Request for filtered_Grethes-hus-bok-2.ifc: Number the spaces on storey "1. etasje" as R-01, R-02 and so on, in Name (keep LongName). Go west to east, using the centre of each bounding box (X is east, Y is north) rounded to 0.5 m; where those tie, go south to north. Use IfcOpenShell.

First a look at what the model holds.

```python
import ifcopenshell
import ifcopenshell.util.element
import ifcopenshell.util.placement

model = ifcopenshell.open("filtered_Grethes-hus-bok-2.ifc")
print(model.schema)
storey = next(s for s in model.by_type("IfcBuildingStorey") if s.Name == "1. etasje")
spaces = [e for e in ifcopenshell.util.element.get_decomposition(storey) if e.is_a("IfcSpace")]
for e in sorted(spaces, key=lambda e: e.id()):
    origin = ifcopenshell.util.placement.get_local_placement(e.ObjectPlacement)[:3, 3]
    print(e.id(), e.Name, e.LongName, origin.round(2) + 0.0, sep=" | ")
```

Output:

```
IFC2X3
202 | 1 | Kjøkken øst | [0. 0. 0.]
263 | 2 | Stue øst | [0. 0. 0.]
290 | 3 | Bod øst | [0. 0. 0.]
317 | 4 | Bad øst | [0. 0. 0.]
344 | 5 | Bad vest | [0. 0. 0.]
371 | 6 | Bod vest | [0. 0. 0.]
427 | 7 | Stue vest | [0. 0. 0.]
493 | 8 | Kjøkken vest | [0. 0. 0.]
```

```python
import ifcopenshell
import ifcopenshell.geom
import ifcopenshell.util.element
import ifcopenshell.util.shape

model = ifcopenshell.open("filtered_Grethes-hus-bok-2.ifc")
settings = ifcopenshell.geom.settings()
settings.set("use-world-coords", True)


def centre(element):
    shape = ifcopenshell.geom.create_shape(settings, element)
    return ifcopenshell.util.shape.get_bbox_centroid(shape.geometry)


storey = next(s for s in model.by_type("IfcBuildingStorey") if s.Name == "1. etasje")
spaces = [e for e in ifcopenshell.util.element.get_decomposition(storey) if e.is_a("IfcSpace")]

# Insertion points can sit at a corner or the storey origin, so sort by the geometry (in metres).
centres = {e: centre(e) for e in spaces}
spaces.sort(key=lambda e: (round(centres[e][0] / 0.5), centres[e][1]))

for i, e in enumerate(spaces, start=1):
    number = f"R-{i:02d}"
    e.Name = number
    print(e.id(), number)

model.write("filtered_Grethes-hus-bok-2_v2.ifc")
```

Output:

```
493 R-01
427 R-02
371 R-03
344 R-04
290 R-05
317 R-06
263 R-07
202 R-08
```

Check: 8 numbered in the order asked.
